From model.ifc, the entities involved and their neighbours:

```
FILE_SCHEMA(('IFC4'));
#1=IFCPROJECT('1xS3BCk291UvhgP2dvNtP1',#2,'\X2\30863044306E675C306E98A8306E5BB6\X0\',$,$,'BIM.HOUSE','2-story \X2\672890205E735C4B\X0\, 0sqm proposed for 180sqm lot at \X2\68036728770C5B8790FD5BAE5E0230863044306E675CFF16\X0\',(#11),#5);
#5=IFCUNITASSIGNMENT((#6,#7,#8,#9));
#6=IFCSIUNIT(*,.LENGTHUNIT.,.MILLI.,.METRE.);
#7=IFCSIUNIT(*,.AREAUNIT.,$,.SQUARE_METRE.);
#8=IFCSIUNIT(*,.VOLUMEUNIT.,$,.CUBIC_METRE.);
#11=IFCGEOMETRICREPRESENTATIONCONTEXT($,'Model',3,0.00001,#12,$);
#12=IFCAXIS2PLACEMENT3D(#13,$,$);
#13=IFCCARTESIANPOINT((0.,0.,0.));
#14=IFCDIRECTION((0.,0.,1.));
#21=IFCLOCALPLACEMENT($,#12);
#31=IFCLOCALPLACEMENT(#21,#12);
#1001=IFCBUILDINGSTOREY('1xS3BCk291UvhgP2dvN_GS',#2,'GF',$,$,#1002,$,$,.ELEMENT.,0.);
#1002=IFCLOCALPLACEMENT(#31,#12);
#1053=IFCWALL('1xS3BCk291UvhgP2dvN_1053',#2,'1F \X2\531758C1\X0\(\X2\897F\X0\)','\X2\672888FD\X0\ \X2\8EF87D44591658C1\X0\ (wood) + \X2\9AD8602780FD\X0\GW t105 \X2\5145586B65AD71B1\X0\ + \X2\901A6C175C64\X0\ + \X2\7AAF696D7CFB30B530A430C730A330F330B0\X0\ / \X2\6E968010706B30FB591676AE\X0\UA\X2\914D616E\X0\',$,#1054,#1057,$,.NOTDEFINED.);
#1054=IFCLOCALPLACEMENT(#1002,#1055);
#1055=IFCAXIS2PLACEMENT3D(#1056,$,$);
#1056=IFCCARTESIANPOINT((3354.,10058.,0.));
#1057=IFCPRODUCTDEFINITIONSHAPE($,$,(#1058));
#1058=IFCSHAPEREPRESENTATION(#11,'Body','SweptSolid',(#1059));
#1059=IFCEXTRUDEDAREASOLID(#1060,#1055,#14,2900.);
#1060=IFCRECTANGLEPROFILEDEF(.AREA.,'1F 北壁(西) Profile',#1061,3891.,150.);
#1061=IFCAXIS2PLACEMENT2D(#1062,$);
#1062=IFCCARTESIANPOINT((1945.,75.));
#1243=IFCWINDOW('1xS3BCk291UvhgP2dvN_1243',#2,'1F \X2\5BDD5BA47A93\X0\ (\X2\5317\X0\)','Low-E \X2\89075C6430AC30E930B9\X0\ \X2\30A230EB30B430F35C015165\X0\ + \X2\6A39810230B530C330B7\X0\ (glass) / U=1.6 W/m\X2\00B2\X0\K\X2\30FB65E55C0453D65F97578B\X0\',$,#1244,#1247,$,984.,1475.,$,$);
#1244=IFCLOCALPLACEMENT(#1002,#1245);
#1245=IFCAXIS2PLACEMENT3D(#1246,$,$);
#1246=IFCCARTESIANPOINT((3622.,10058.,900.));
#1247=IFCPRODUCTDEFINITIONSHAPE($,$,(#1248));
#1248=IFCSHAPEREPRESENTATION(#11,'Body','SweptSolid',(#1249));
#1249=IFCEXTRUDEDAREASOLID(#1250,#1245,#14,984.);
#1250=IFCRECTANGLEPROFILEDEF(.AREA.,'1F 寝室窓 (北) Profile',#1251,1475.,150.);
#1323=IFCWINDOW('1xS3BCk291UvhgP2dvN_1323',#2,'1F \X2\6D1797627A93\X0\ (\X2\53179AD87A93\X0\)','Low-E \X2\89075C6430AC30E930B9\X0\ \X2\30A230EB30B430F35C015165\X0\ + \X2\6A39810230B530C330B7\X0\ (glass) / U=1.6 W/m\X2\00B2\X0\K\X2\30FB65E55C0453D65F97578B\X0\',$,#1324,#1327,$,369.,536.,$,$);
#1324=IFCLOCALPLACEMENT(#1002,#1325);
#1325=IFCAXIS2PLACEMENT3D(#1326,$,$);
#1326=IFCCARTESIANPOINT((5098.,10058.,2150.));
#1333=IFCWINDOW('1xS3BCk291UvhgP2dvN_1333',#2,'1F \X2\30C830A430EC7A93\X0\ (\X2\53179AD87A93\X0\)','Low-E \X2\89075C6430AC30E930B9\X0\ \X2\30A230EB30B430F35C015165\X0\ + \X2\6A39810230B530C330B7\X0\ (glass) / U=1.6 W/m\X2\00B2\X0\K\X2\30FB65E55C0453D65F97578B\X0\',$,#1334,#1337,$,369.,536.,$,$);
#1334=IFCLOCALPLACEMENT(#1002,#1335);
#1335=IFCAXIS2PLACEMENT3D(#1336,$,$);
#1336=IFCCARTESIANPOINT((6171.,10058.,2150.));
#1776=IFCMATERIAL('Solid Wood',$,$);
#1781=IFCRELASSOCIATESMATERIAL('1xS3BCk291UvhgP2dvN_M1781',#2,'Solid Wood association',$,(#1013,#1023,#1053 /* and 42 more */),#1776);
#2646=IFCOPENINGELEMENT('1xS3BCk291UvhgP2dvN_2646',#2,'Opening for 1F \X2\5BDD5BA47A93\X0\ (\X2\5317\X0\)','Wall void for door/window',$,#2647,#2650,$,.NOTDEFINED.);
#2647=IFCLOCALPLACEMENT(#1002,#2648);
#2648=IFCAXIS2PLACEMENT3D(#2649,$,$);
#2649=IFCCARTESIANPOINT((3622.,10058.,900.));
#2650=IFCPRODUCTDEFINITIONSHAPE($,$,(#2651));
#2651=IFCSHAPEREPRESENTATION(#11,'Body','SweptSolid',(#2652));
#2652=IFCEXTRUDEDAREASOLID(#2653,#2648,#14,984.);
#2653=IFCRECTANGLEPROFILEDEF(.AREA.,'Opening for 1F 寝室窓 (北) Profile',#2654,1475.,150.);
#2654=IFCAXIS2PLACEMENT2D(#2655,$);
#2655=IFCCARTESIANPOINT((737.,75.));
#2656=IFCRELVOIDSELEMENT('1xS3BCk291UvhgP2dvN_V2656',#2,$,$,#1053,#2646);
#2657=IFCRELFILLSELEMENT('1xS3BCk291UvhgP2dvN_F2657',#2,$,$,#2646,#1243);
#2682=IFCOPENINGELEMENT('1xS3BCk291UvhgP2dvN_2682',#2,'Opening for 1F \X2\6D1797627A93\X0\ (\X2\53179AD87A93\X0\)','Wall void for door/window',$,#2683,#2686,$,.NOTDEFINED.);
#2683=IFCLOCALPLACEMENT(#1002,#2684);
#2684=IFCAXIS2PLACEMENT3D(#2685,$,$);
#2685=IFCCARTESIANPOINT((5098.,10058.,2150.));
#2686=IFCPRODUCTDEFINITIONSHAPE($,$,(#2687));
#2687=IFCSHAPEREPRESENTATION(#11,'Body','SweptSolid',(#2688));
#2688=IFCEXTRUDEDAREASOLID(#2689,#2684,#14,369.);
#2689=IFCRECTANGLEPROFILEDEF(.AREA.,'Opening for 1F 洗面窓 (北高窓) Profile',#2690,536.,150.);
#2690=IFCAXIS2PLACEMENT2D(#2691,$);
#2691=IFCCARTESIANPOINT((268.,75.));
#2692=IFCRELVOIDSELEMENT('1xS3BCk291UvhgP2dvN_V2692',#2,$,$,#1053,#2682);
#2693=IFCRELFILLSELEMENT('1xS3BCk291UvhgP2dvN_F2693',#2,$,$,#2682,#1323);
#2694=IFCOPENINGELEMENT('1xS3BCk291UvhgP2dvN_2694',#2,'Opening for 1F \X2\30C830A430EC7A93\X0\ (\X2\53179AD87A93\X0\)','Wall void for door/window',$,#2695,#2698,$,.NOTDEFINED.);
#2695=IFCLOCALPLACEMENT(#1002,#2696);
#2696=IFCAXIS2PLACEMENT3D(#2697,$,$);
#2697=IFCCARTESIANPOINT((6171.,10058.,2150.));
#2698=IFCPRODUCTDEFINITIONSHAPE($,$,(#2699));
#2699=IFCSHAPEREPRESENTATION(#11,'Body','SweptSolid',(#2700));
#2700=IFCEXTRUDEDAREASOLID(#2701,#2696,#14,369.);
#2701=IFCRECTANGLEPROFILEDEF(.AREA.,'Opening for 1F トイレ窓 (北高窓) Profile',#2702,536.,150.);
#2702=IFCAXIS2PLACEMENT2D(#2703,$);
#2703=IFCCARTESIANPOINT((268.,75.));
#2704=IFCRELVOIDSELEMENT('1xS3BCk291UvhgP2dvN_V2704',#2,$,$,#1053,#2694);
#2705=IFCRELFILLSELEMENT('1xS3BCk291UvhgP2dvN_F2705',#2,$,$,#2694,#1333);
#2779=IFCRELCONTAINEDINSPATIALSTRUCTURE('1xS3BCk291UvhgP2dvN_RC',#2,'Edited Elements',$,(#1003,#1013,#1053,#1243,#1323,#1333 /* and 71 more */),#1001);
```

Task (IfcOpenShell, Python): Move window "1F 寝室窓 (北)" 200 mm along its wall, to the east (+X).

```python
import ifcopenshell
import ifcopenshell.api.geometry
import ifcopenshell.util.placement

model = ifcopenshell.open("model.ifc")

window = model.by_id(1243)
opening = window.FillsVoids[0].RelatingOpeningElement
wall = opening.VoidsElements[0].RelatingBuildingElement

wall_matrix = ifcopenshell.util.placement.get_local_placement(wall.ObjectPlacement)
shift = wall_matrix[:3, 0] * 200.0
before = ifcopenshell.util.placement.get_local_placement(window.ObjectPlacement)[:3, 3].copy()

# The window is not placed relative to its opening, so move both.
for product in (opening, window):
    matrix = ifcopenshell.util.placement.get_local_placement(product.ObjectPlacement)
    matrix[:3, 3] += shift
    ifcopenshell.api.geometry.edit_object_placement(model, product=product, matrix=matrix, is_si=False)

after = ifcopenshell.util.placement.get_local_placement(window.ObjectPlacement)[:3, 3]
print("window moved by", (after - before).round(3) + 0.0)

model.write("model_v2.ifc")
```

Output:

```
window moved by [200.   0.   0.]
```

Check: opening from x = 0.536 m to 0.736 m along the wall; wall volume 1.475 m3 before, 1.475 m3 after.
